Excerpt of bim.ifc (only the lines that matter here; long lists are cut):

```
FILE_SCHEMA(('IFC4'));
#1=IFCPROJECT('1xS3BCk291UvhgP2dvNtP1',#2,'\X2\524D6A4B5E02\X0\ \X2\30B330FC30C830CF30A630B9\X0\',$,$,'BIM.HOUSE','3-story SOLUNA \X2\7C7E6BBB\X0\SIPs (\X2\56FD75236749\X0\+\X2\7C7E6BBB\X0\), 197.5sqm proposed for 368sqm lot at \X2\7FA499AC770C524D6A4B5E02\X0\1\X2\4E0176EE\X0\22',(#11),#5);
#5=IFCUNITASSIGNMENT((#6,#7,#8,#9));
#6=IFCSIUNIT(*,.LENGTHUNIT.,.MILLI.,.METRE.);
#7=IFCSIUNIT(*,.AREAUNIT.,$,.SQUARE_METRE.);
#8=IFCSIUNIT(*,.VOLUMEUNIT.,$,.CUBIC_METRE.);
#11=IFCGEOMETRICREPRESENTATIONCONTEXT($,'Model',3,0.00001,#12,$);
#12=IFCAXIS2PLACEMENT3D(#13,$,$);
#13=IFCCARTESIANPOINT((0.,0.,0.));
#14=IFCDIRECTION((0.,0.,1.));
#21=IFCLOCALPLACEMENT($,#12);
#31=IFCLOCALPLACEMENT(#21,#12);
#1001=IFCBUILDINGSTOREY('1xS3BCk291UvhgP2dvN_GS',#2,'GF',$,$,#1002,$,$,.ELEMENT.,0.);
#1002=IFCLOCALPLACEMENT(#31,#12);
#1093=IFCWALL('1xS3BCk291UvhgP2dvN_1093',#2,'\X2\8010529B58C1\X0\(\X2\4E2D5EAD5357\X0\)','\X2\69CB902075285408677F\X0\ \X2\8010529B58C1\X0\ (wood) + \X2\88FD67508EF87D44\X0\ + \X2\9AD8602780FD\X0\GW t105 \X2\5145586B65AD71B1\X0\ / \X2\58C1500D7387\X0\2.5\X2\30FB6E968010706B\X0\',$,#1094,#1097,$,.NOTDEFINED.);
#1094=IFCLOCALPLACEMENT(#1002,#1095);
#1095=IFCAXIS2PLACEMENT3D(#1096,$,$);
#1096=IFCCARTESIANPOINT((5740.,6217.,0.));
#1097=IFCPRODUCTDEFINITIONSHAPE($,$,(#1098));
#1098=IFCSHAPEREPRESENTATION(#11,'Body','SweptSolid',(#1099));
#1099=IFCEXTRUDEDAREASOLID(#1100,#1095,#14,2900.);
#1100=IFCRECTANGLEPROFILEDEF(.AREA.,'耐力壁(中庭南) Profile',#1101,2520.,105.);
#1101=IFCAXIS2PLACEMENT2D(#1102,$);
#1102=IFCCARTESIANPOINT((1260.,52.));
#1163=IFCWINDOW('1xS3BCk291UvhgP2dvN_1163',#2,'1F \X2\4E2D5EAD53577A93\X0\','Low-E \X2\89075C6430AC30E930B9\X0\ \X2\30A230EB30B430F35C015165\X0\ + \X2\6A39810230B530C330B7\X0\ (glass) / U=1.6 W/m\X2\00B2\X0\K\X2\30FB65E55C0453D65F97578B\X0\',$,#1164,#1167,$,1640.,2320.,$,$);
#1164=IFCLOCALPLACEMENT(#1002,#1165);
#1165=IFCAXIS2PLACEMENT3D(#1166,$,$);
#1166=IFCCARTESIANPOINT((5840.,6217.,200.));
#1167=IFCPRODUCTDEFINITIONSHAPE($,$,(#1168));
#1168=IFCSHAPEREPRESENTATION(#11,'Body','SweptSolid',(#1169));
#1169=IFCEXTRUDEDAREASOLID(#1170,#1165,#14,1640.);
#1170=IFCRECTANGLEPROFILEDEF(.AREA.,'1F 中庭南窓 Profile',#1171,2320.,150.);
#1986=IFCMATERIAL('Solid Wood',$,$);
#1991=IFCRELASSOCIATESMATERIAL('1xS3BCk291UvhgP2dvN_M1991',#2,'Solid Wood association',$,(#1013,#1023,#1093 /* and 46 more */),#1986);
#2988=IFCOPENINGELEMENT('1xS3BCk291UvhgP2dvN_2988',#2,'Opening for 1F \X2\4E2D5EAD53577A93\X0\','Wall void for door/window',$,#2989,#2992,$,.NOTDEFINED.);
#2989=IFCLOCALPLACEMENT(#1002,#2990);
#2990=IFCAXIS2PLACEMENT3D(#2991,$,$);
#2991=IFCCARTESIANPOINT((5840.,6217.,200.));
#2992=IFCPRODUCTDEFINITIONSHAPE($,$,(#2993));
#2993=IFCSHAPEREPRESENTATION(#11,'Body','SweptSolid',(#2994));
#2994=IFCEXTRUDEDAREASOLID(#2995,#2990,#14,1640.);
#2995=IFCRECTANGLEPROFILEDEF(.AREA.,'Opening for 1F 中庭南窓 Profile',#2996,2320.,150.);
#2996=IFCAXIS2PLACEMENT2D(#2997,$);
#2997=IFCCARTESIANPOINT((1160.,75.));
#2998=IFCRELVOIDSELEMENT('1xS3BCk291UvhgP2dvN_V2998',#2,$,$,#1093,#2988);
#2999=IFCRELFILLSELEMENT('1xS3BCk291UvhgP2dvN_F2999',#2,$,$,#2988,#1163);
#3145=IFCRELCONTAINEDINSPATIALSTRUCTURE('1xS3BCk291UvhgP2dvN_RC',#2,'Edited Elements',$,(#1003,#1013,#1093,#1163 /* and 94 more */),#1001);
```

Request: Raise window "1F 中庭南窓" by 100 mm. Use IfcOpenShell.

```python
import numpy as np
import ifcopenshell
import ifcopenshell.api.geometry
import ifcopenshell.util.placement
import ifcopenshell.util.unit

model = ifcopenshell.open("bim.ifc")
unit_scale = ifcopenshell.util.unit.calculate_unit_scale(model)

window = model.by_guid("1xS3BCk291UvhgP2dvN_1163")
opening = window.FillsVoids[0].RelatingOpeningElement
dz = 100.0

shift = np.array([0.0, 0.0, dz])
# The window is not placed relative to its opening, so move both.
for product in (opening, window):
    matrix = ifcopenshell.util.placement.get_local_placement(product.ObjectPlacement)
    matrix[:3, 3] += shift
    ifcopenshell.api.geometry.edit_object_placement(model, product=product, matrix=matrix, is_si=False)

print(f"moved by {dz * unit_scale:+.3f} m")

model.write("bim_edited.ifc")
```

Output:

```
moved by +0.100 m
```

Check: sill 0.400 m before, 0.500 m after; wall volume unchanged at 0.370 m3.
